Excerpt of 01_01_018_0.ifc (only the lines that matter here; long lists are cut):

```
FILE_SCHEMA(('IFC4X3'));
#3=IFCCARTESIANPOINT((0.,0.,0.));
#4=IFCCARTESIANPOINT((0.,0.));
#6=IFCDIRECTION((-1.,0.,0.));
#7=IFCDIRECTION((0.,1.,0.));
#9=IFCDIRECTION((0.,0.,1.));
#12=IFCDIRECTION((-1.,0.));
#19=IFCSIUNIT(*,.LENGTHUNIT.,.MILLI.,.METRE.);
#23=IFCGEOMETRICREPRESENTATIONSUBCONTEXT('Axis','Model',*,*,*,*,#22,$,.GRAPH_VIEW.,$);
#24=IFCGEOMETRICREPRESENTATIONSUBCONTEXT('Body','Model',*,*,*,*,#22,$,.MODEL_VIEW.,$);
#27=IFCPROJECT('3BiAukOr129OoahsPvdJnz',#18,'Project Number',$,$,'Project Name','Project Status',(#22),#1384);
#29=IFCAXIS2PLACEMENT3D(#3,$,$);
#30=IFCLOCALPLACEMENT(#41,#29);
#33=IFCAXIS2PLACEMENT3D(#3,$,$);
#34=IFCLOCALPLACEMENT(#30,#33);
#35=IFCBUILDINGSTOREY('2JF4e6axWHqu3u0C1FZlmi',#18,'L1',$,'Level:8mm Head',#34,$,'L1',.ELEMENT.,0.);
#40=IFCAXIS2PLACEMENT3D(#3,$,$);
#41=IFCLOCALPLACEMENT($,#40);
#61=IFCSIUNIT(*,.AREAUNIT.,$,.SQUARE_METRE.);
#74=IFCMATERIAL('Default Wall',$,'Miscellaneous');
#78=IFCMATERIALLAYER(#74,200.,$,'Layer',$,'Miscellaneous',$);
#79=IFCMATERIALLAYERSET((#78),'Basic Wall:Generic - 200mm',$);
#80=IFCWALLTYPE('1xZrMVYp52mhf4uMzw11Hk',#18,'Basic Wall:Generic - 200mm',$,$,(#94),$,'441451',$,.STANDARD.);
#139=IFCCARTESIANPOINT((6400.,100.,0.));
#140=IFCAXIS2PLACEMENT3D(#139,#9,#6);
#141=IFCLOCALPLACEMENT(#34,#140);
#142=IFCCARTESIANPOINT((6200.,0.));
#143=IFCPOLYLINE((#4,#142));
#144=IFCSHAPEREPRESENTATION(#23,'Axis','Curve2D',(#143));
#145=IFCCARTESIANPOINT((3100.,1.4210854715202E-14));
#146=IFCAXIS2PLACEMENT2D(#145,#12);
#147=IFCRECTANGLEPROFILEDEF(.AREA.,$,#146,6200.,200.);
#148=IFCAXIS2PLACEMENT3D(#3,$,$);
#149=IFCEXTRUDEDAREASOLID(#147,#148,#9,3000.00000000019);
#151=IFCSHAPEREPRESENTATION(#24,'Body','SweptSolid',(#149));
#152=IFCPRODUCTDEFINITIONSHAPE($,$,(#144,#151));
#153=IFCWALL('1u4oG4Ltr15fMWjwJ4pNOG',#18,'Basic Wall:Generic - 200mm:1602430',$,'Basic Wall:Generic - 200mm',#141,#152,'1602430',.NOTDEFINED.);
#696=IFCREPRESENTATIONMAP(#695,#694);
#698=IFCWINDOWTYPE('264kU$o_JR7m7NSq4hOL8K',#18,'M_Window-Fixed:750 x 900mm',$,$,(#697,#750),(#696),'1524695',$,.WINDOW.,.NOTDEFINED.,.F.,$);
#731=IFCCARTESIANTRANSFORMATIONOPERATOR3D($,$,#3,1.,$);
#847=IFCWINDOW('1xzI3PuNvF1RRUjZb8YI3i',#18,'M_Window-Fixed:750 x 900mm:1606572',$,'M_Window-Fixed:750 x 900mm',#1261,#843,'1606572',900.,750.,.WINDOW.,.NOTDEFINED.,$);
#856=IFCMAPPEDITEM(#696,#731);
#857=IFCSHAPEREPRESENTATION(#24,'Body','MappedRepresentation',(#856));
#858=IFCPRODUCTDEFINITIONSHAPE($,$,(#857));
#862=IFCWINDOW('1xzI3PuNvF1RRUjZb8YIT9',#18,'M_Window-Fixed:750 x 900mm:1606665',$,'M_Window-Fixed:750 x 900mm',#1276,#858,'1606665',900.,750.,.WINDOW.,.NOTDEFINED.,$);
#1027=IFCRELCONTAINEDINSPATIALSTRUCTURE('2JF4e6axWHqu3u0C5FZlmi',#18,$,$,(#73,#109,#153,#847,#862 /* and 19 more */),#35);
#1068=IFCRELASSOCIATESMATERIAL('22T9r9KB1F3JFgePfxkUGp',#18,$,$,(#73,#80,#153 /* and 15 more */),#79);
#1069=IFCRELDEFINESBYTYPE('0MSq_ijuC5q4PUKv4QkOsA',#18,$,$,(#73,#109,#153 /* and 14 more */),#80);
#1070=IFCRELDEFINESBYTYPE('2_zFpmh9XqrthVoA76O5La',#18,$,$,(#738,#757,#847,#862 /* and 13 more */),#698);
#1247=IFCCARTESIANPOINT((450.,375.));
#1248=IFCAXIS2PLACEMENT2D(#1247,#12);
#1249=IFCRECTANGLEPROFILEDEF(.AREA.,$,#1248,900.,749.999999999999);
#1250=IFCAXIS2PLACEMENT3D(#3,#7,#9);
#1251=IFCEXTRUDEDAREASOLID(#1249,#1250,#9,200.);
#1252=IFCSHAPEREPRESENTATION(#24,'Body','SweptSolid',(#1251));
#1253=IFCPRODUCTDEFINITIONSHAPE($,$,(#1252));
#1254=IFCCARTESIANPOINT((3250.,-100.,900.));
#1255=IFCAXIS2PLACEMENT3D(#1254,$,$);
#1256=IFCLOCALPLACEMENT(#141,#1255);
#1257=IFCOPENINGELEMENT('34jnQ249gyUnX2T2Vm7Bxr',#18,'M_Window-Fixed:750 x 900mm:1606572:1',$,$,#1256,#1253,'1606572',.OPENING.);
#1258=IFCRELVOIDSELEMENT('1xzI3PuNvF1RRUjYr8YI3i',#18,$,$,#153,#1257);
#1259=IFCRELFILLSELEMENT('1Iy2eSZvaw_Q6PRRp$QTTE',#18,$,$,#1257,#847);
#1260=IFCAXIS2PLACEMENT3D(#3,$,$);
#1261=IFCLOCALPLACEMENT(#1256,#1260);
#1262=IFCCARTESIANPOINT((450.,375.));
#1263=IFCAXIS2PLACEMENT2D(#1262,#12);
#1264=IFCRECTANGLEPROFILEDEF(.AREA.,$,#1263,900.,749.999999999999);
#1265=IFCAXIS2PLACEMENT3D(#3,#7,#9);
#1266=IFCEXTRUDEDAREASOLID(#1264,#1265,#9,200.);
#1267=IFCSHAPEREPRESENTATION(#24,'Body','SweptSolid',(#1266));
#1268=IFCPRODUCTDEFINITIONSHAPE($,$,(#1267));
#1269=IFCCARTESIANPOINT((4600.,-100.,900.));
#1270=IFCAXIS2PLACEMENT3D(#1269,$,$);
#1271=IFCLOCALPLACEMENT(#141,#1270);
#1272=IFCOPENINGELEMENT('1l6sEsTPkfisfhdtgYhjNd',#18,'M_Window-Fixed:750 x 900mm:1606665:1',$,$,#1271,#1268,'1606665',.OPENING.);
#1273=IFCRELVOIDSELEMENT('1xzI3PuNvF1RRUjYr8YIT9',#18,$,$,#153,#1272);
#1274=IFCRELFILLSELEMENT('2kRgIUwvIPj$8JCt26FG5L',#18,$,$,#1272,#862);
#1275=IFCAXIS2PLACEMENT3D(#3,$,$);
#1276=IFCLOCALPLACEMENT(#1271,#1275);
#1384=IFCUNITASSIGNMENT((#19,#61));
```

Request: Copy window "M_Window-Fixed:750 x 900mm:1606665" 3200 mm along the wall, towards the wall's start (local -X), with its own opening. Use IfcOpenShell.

```python
import ifcopenshell
import ifcopenshell.api.feature
import ifcopenshell.api.geometry
import ifcopenshell.api.root
import ifcopenshell.geom
import ifcopenshell.util.element
import ifcopenshell.util.placement
import ifcopenshell.util.shape
import ifcopenshell.util.unit

model = ifcopenshell.open("01_01_018_0.ifc")
unit_scale = ifcopenshell.util.unit.calculate_unit_scale(model)
settings = ifcopenshell.geom.settings()


def volume(element):
    """Net volume in cubic metres, openings subtracted."""
    shape = ifcopenshell.geom.create_shape(settings, element)
    return ifcopenshell.util.shape.get_volume(shape.geometry)


def reuse_history(source, copy):
    """copy_class also copies each property set's owner history, people and application; keep the originals."""
    for rel in copy.IsDefinedBy:
        if rel.is_a("IfcRelDefinesByProperties") and (history := rel.RelatingPropertyDefinition.OwnerHistory):
            rel.RelatingPropertyDefinition.OwnerHistory = source.OwnerHistory
            ifcopenshell.util.element.remove_deep2(model, history)


window = model.by_guid("1xzI3PuNvF1RRUjZb8YIT9")
opening = window.FillsVoids[0].RelatingOpeningElement
wall = opening.VoidsElements[0].RelatingBuildingElement
before = volume(wall)
shift = ifcopenshell.util.placement.get_local_placement(wall.ObjectPlacement)[:3, 0] * -3.2 / unit_scale

# copy_class copies the void relationship, type, container and properties, but no geometry.
new_opening = ifcopenshell.api.root.copy_class(model, product=opening)
new_opening.Representation = ifcopenshell.util.element.copy_deep(
    model, opening.Representation, exclude=["IfcGeometricRepresentationContext", "IfcRepresentationMap"]
)
new_opening.Name = "M_Window-Fixed:750 x 900mm"
new_opening.Tag = None
new_window = ifcopenshell.api.root.copy_class(model, product=window)
new_window.Representation = ifcopenshell.util.element.copy_deep(
    model, window.Representation, exclude=["IfcGeometricRepresentationContext", "IfcRepresentationMap"]
)
new_window.Name = "M_Window-Fixed:750 x 900mm"
new_window.Tag = None
reuse_history(window, new_window)
ifcopenshell.api.feature.add_filling(model, opening=new_opening, element=new_window)

for old, new in ((opening, new_opening), (window, new_window)):
    matrix = ifcopenshell.util.placement.get_local_placement(old.ObjectPlacement)
    matrix[:3, 3] += shift
    ifcopenshell.api.geometry.edit_object_placement(model, product=new, matrix=matrix, is_si=False)

after = volume(wall)

print(f"wall volume {before:.3f} -> {after:.3f} m3")

model.write("01_01_018_0_rev.ifc")
```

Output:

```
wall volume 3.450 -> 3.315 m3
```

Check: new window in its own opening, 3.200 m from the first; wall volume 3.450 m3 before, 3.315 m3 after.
